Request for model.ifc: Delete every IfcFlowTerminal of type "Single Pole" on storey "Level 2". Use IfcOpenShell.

First a look at what the model holds.

```python
import ifcopenshell
import ifcopenshell.util.element

model = ifcopenshell.open("model.ifc")
print(model.schema)
storey = next(s for s in model.by_type("IfcBuildingStorey") if s.Name == "Level 2")
terminals = [e for e in ifcopenshell.util.element.get_decomposition(storey) if e.is_a("IfcFlowTerminal")]
seen = {}
for e in terminals:
    element_type = ifcopenshell.util.element.get_type(e)
    name = element_type.Name if element_type not in (None, e) else None
    seen[name] = seen.get(name, 0) + 1
for name, count in sorted(seen.items(), key=str):
    print(count, "x", name)
```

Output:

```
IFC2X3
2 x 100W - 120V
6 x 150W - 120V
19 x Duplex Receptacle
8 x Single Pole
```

```python
import ifcopenshell
import ifcopenshell.api.root
import ifcopenshell.util.element

model = ifcopenshell.open("model.ifc")

storey = next(s for s in model.by_type("IfcBuildingStorey") if s.Name == "Level 2")
terminals = [e for e in ifcopenshell.util.element.get_decomposition(storey) if e.is_a("IfcFlowTerminal")]
targets = [e for e in terminals if (t := ifcopenshell.util.element.get_type(e)) not in (None, e) and t.Name == "Single Pole"]

for e in targets:
    ifcopenshell.api.root.remove_product(model, product=e)
print(len(targets), "removed")

model.write("model_updated.ifc")
```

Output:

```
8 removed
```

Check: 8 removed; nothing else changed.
